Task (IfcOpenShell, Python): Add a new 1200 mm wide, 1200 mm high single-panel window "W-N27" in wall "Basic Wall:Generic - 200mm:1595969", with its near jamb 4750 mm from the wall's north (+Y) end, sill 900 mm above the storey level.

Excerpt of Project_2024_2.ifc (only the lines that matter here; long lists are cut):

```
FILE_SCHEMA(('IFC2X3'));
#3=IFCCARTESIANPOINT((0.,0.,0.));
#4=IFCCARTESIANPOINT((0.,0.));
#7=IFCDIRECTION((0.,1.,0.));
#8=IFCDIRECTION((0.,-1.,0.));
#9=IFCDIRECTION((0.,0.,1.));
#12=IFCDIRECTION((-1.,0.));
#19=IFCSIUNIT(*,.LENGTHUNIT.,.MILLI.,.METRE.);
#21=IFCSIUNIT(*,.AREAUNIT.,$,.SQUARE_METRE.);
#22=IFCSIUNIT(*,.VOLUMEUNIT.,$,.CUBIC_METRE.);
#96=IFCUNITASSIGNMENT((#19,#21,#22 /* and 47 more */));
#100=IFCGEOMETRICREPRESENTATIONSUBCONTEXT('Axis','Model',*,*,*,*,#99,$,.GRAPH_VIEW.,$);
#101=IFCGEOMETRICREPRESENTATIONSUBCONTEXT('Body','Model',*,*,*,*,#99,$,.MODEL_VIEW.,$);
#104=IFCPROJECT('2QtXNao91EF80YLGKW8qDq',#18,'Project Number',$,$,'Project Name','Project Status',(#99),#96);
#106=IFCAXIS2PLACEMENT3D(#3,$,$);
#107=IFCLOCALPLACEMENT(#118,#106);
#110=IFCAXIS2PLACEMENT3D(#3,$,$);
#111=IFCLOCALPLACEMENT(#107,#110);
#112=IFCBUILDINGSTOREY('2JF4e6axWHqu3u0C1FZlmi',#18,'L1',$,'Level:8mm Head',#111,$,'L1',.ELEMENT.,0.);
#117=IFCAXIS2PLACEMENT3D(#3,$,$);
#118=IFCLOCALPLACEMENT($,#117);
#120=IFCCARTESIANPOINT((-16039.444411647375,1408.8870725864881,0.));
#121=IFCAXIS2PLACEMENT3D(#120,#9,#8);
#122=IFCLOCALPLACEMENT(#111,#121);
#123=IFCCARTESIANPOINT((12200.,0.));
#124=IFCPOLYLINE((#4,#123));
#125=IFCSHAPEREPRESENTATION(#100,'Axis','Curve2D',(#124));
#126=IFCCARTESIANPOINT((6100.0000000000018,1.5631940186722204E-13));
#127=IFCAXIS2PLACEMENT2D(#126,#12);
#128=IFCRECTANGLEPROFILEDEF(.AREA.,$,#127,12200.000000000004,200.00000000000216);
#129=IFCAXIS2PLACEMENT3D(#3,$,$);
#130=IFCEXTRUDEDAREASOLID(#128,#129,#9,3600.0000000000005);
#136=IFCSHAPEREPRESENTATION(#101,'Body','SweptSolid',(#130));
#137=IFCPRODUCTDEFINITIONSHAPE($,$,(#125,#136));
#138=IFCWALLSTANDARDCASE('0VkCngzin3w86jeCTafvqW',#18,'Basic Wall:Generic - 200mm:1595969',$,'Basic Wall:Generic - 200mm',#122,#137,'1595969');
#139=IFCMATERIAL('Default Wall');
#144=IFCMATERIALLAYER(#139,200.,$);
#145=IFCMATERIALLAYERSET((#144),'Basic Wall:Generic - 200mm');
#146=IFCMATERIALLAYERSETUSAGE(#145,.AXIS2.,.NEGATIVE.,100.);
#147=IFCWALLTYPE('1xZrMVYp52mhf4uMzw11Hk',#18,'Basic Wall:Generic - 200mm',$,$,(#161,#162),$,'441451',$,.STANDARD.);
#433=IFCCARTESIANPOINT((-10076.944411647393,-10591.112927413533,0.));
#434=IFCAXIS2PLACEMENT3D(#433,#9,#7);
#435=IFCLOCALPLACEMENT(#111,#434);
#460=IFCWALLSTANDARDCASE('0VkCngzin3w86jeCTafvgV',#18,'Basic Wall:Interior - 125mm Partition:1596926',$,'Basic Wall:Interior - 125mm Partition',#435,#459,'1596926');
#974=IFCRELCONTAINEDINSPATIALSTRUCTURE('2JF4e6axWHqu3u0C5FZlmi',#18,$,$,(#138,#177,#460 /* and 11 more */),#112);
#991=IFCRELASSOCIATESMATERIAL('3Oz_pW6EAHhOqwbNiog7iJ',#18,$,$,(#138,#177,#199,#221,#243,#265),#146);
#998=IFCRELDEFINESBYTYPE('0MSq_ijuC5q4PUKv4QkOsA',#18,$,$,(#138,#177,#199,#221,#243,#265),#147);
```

```python
import numpy as np
import ifcopenshell
import ifcopenshell.api.feature
import ifcopenshell.api.geometry
import ifcopenshell.api.root
import ifcopenshell.api.spatial
import ifcopenshell.api.type
import ifcopenshell.geom
import ifcopenshell.util.element
import ifcopenshell.util.placement
import ifcopenshell.util.representation
import ifcopenshell.util.shape
import ifcopenshell.util.unit

model = ifcopenshell.open("Project_2024_2.ifc")
unit_scale = ifcopenshell.util.unit.calculate_unit_scale(model)
settings = ifcopenshell.geom.settings()


def volume(element):
    """Net volume in cubic metres, openings subtracted."""
    shape = ifcopenshell.geom.create_shape(settings, element)
    return ifcopenshell.util.shape.get_volume(shape.geometry)


wall = model.by_guid("0VkCngzin3w86jeCTafvqW")
storey = ifcopenshell.util.element.get_container(wall, ifc_class="IfcBuildingStorey")
context = ifcopenshell.util.representation.get_context(model, "Model", "Body", "MODEL_VIEW")
before = volume(wall)

width, height, from_end, sill = 1.2, 1.2, 4.75, 0.9  # metres

# The wall runs along its own X axis, and the end named is its -X end.
wall_shape = ifcopenshell.geom.create_shape(settings, wall)
x, y, z = ifcopenshell.util.shape.get_vertices(wall_shape.geometry).T
start = x.min() + from_end
face, thickness = float(y.min()), float(y.max() - y.min())
wall_matrix = ifcopenshell.util.placement.get_local_placement(wall.ObjectPlacement)
level = ifcopenshell.util.placement.get_local_placement(storey.ObjectPlacement)[2, 3]


def in_wall(x, y):
    """Placement at x, y metres in the wall's axes, at sill height."""
    matrix = wall_matrix.copy()
    matrix[:, 3] = wall_matrix @ np.array([x / unit_scale, y / unit_scale, 0.0, 1.0])
    matrix[2, 3] = level + sill / unit_scale
    return matrix


# Opening: a box that overshoots both wall faces by 50 mm.
opening = ifcopenshell.api.root.create_entity(model, ifc_class="IfcOpeningElement")
box = ifcopenshell.api.geometry.add_wall_representation(
    model, context=context, length=width, height=height, thickness=thickness + 0.1
)
ifcopenshell.api.geometry.assign_representation(model, product=opening, representation=box)
ifcopenshell.api.geometry.edit_object_placement(model, product=opening, matrix=in_wall(start, face - 0.05), is_si=False)
ifcopenshell.api.feature.add_feature(model, feature=opening, element=wall)

window = ifcopenshell.api.root.create_entity(model, ifc_class="IfcWindow", name="W-N27")
window.OverallWidth, window.OverallHeight = width / unit_scale, height / unit_scale
body = ifcopenshell.api.geometry.add_window_representation(
    model,
    context=context,
    overall_width=window.OverallWidth,
    overall_height=window.OverallHeight,
    partition_type="SINGLE_PANEL",
)
ifcopenshell.api.geometry.assign_representation(model, product=window, representation=body)
ifcopenshell.api.spatial.assign_container(model, products=[window], relating_structure=storey)
fills = ifcopenshell.api.feature.add_filling(model, opening=opening, element=window)
fills.OwnerHistory = window.OwnerHistory  # required in IFC2X3

# IFC2X3 keeps the operation on the window style.
style = ifcopenshell.api.root.create_entity(model, ifc_class="IfcWindowStyle", name="W-N27")
style.OperationType, style.ConstructionType = "SINGLE_PANEL", "NOTDEFINED"
style.ParameterTakesPrecedence = style.Sizeable = False
ifcopenshell.api.type.assign_type(model, related_objects=[window], relating_type=style)

# Centre the window in the wall's thickness.
ifcopenshell.api.geometry.edit_object_placement(model, product=window, matrix=in_wall(start, face), is_si=False)
window_shape = ifcopenshell.geom.create_shape(settings, window)
depth = ifcopenshell.util.shape.get_vertices(window_shape.geometry)[:, 1]
offset = face + thickness / 2 - (depth.min() + depth.max()) / 2
ifcopenshell.api.geometry.edit_object_placement(model, product=window, matrix=in_wall(start, offset), is_si=False)

after = volume(wall)

print(f"wall volume {before:.3f} -> {after:.3f} m3")

model.write("Project_2024_2_rev.ifc")
```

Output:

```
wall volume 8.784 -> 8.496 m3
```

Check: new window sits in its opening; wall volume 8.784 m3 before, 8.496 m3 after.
